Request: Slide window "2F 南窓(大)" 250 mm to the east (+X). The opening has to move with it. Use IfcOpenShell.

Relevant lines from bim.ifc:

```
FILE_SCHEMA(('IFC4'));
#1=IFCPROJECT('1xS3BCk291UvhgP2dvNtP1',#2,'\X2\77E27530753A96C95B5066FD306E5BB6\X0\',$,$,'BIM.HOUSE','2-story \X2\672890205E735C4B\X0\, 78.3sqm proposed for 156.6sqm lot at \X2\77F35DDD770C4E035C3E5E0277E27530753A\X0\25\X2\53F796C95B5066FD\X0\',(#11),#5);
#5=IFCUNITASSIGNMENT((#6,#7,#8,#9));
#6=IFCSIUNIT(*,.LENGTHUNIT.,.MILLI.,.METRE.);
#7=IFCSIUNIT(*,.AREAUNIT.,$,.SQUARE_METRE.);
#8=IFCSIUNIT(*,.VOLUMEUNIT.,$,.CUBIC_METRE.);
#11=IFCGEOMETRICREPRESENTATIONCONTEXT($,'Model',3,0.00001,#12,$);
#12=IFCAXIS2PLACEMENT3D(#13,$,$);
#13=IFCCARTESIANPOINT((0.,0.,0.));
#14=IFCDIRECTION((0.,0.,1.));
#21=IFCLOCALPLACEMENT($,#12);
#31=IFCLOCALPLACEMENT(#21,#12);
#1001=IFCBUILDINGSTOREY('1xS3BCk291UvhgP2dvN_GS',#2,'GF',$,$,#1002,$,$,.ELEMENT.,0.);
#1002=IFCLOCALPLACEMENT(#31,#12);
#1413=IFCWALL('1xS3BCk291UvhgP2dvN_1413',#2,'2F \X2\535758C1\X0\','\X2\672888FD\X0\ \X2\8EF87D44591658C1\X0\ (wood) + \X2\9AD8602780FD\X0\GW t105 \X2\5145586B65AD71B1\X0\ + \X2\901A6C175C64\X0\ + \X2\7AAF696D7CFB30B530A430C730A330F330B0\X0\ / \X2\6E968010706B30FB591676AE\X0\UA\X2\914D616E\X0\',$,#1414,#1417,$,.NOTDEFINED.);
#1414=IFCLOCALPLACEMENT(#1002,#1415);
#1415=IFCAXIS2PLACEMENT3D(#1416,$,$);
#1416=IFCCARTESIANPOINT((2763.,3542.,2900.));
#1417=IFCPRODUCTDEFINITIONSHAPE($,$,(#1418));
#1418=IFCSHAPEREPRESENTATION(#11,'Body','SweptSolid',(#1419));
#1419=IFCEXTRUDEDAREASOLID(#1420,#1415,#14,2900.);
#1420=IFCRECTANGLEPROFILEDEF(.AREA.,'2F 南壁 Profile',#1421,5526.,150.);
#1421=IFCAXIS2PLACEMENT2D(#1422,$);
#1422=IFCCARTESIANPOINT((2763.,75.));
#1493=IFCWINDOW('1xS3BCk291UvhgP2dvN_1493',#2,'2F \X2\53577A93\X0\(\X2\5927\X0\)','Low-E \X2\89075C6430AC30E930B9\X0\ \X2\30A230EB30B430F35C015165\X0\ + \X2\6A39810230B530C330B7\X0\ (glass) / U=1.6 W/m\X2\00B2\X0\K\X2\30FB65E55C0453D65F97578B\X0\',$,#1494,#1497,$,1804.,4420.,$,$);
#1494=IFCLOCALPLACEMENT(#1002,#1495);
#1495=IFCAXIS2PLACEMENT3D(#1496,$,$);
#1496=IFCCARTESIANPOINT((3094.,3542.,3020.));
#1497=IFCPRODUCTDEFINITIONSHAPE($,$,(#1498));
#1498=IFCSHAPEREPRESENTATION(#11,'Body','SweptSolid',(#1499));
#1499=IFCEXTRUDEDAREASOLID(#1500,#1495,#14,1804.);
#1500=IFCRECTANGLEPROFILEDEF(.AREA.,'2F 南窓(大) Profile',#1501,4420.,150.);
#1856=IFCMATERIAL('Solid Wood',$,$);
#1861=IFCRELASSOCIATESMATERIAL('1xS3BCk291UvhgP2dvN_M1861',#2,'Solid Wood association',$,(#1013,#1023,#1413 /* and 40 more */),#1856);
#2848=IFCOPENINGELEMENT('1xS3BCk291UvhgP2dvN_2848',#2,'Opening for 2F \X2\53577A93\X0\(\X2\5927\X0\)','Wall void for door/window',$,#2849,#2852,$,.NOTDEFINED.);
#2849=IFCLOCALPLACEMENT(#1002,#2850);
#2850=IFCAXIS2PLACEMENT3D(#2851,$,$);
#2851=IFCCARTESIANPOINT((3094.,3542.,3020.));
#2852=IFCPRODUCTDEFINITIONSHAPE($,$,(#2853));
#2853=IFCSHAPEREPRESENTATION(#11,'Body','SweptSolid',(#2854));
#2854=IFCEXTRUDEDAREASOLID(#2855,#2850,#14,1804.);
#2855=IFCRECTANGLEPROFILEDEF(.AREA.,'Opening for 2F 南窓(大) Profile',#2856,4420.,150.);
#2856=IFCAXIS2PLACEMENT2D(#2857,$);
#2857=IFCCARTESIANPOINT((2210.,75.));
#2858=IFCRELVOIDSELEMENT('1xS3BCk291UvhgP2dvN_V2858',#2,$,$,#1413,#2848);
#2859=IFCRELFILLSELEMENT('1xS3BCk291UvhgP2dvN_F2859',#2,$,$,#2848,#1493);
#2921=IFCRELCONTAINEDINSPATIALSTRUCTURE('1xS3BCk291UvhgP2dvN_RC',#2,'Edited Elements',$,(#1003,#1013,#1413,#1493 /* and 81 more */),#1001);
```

```python
import ifcopenshell
import ifcopenshell.api.geometry
import ifcopenshell.util.placement
import ifcopenshell.util.unit

model = ifcopenshell.open("bim.ifc")
unit_scale = ifcopenshell.util.unit.calculate_unit_scale(model)

window = model.by_guid("1xS3BCk291UvhgP2dvN_1493")
opening = window.FillsVoids[0].RelatingOpeningElement
wall = opening.VoidsElements[0].RelatingBuildingElement

wall_matrix = ifcopenshell.util.placement.get_local_placement(wall.ObjectPlacement)
shift = wall_matrix[:3, 0] * 0.25 / unit_scale
before = ifcopenshell.util.placement.get_local_placement(window.ObjectPlacement)[:3, 3].copy()

# The window is not placed relative to its opening, so move both.
for product in (opening, window):
    matrix = ifcopenshell.util.placement.get_local_placement(product.ObjectPlacement)
    matrix[:3, 3] += shift
    ifcopenshell.api.geometry.edit_object_placement(model, product=product, matrix=matrix, is_si=False)

after = ifcopenshell.util.placement.get_local_placement(window.ObjectPlacement)[:3, 3]
print("window moved by", (after - before).round(3) + 0.0)

model.write("bim-out.ifc")
```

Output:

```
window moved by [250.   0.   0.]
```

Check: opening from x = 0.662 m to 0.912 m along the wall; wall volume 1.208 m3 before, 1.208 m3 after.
